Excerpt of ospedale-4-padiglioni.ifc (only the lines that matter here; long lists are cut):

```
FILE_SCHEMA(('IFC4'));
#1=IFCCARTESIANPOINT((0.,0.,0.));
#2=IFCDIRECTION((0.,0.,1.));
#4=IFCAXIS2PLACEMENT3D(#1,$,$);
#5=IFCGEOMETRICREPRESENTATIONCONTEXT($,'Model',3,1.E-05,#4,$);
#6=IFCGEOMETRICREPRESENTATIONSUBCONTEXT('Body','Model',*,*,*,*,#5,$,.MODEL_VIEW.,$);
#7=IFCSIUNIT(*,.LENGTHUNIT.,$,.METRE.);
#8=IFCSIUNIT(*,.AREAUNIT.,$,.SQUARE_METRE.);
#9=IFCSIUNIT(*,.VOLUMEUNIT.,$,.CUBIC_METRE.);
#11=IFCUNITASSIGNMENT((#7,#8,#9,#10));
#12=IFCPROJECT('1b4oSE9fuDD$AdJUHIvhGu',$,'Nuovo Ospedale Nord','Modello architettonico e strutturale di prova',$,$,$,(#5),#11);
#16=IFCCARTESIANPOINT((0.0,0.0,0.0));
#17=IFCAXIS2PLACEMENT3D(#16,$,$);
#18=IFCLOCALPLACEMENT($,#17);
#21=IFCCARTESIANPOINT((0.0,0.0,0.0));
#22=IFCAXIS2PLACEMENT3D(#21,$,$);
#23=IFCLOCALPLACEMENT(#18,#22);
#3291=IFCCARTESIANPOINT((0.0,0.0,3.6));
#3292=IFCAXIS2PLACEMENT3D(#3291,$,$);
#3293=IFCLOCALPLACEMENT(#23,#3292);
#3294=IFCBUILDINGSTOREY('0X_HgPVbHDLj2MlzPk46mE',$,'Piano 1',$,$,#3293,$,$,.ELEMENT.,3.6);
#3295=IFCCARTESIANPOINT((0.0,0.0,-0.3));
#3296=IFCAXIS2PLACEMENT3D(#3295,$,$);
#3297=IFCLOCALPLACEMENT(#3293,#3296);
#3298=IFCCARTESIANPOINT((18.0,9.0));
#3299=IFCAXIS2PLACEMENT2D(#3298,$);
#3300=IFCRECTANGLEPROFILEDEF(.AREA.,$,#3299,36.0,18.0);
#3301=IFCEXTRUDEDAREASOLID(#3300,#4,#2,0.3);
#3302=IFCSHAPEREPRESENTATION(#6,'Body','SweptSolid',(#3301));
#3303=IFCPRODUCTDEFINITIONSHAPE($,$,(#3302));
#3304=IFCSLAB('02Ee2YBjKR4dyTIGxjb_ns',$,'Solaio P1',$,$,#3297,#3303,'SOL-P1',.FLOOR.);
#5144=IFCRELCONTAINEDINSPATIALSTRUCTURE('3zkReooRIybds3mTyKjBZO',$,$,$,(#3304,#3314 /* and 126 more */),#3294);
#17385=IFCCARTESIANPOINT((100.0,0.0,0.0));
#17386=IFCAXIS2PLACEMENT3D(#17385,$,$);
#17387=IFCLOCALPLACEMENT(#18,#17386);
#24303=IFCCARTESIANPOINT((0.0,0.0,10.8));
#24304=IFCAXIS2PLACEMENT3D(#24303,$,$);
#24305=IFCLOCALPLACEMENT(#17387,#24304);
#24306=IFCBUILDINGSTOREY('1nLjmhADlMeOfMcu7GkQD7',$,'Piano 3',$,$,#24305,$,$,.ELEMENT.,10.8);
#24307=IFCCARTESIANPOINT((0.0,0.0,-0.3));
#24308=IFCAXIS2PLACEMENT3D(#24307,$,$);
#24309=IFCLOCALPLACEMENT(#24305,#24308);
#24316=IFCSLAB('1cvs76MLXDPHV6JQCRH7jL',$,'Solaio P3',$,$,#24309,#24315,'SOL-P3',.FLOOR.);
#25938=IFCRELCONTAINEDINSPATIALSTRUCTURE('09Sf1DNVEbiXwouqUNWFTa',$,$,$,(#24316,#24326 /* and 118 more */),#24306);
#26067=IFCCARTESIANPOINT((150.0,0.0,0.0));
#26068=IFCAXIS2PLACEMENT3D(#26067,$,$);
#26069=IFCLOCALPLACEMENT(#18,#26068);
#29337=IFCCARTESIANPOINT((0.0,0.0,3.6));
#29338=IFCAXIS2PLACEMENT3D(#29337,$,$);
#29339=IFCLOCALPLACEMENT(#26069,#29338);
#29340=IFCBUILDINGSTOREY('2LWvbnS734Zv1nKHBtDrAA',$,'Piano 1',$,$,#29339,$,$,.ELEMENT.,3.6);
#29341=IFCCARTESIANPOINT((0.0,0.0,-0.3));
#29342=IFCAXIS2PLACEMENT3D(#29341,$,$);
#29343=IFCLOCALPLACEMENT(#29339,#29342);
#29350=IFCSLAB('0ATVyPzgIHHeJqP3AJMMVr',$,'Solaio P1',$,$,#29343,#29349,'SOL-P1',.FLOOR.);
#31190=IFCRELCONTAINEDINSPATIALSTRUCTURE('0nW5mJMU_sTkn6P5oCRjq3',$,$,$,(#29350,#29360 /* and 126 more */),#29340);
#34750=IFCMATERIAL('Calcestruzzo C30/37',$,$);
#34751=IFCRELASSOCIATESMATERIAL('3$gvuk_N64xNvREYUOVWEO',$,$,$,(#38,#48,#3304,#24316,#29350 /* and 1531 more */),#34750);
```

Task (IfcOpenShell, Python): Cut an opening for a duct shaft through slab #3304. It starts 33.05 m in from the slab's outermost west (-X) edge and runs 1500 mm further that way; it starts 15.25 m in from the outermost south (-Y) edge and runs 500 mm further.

```python
import numpy as np
import ifcopenshell
import ifcopenshell.api.feature
import ifcopenshell.api.geometry
import ifcopenshell.api.root
import ifcopenshell.geom
import ifcopenshell.util.placement
import ifcopenshell.util.representation
import ifcopenshell.util.shape
import ifcopenshell.util.unit

model = ifcopenshell.open("ospedale-4-padiglioni.ifc")
unit_scale = ifcopenshell.util.unit.calculate_unit_scale(model)
settings = ifcopenshell.geom.settings()


def volume(element):
    """Net volume in cubic metres, openings subtracted."""
    shape = ifcopenshell.geom.create_shape(settings, element)
    return ifcopenshell.util.shape.get_volume(shape.geometry)


slab = model.by_id(3304)
before = volume(slab)

# Extent in the slab's own axes, in metres. The edges named are its -X and -Y sides.
slab_shape = ifcopenshell.geom.create_shape(settings, slab)
vertices = ifcopenshell.util.shape.get_vertices(slab_shape.geometry)
x_min, y_min, bottom = vertices.min(axis=0)
top = vertices[:, 2].max()

opening = ifcopenshell.api.root.create_entity(model, ifc_class="IfcOpeningElement", name="Duct shaft opening", predefined_type="OPENING")
context = ifcopenshell.util.representation.get_context(model, "Model", "Body", "MODEL_VIEW")
width, depth = 1.5, 0.5
outline = [(0.0, 0.0), (width, 0.0), (width, depth), (0.0, depth), (0.0, 0.0)]
# Overshoot both faces by 50 mm so the cut is clean.
shape = ifcopenshell.api.geometry.add_slab_representation(
    model, context=context, depth=top - bottom + 0.1, polyline=outline
)
ifcopenshell.api.geometry.assign_representation(model, product=opening, representation=shape)

matrix = ifcopenshell.util.placement.get_local_placement(slab.ObjectPlacement)
matrix[:, 3] = matrix @ np.append(np.array([x_min + 33.05, y_min + 15.25, bottom - 0.05]) / unit_scale, 1.0)
ifcopenshell.api.geometry.edit_object_placement(model, product=opening, matrix=matrix, is_si=False)
ifcopenshell.api.feature.add_feature(model, feature=opening, element=slab)

after = volume(slab)

print(f"slab volume {before:.3f} -> {after:.3f} m3")

model.write("ospedale-4-padiglioni_v2.ifc")
```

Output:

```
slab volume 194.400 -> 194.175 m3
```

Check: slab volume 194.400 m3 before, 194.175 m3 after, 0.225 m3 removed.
